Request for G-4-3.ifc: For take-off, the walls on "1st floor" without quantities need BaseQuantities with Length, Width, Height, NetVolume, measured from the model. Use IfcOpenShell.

First a look at what the model holds.

```python
import ifcopenshell
import ifcopenshell.util.element
import ifcopenshell.util.unit

model = ifcopenshell.open("G-4-3.ifc")
print(model.schema)
for unit_type in ("LENGTHUNIT", "AREAUNIT", "VOLUMEUNIT"):
    print(unit_type, ifcopenshell.util.unit.calculate_unit_scale(model, unit_type))
storey = next(s for s in model.by_type("IfcBuildingStorey") if s.Name == "1st floor")
walls = [e for e in ifcopenshell.util.element.get_decomposition(storey) if e.is_a("IfcWall")]
for e in sorted(walls, key=lambda e: e.id()):
    print(e.id(), e.is_a(), e.Name, list(ifcopenshell.util.element.get_psets(e, qtos_only=True)), sep=" | ")
```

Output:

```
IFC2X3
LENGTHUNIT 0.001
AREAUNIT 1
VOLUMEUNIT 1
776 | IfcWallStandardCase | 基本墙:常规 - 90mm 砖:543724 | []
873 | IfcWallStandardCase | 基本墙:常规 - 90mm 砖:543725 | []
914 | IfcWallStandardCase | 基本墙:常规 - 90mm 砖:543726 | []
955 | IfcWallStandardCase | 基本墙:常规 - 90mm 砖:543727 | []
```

```python
import ifcopenshell
import ifcopenshell.api.pset
import ifcopenshell.geom
import ifcopenshell.util.element
import ifcopenshell.util.shape
import ifcopenshell.util.unit

model = ifcopenshell.open("G-4-3.ifc")
unit_scale = ifcopenshell.util.unit.calculate_unit_scale(model)
volume_scale = ifcopenshell.util.unit.calculate_unit_scale(model, "VOLUMEUNIT")
settings = ifcopenshell.geom.settings()

storey = next(s for s in model.by_type("IfcBuildingStorey") if s.Name == "1st floor")
walls = [e for e in ifcopenshell.util.element.get_decomposition(storey) if e.is_a("IfcWall")]

for e in sorted(walls, key=lambda e: e.id()):
    if ifcopenshell.util.element.get_psets(e, qtos_only=True, should_inherit=False):
        continue
    # Geometry comes back in metres, in the element's own axes.
    shape = ifcopenshell.geom.create_shape(settings, e)
    values = {
        "Length": ifcopenshell.util.shape.get_x(shape.geometry) / unit_scale,
        "Width": ifcopenshell.util.shape.get_y(shape.geometry) / unit_scale,
        "Height": ifcopenshell.util.shape.get_z(shape.geometry) / unit_scale,
        "NetVolume": ifcopenshell.util.shape.get_volume(shape.geometry) / volume_scale,
    }
    qto = ifcopenshell.api.pset.add_qto(model, product=e, name="BaseQuantities")
    ifcopenshell.api.pset.edit_qto(model, qto=qto, properties=values)
    print(e.id(), {k: round(v, 3) for k, v in values.items()})

model.write("G-4-3-out.ifc")
```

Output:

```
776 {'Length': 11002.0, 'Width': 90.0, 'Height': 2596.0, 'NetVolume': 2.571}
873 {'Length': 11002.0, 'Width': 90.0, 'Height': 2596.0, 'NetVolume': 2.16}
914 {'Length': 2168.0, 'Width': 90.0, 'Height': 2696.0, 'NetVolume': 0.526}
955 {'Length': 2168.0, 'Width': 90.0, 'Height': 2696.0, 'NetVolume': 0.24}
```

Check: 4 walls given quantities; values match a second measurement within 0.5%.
